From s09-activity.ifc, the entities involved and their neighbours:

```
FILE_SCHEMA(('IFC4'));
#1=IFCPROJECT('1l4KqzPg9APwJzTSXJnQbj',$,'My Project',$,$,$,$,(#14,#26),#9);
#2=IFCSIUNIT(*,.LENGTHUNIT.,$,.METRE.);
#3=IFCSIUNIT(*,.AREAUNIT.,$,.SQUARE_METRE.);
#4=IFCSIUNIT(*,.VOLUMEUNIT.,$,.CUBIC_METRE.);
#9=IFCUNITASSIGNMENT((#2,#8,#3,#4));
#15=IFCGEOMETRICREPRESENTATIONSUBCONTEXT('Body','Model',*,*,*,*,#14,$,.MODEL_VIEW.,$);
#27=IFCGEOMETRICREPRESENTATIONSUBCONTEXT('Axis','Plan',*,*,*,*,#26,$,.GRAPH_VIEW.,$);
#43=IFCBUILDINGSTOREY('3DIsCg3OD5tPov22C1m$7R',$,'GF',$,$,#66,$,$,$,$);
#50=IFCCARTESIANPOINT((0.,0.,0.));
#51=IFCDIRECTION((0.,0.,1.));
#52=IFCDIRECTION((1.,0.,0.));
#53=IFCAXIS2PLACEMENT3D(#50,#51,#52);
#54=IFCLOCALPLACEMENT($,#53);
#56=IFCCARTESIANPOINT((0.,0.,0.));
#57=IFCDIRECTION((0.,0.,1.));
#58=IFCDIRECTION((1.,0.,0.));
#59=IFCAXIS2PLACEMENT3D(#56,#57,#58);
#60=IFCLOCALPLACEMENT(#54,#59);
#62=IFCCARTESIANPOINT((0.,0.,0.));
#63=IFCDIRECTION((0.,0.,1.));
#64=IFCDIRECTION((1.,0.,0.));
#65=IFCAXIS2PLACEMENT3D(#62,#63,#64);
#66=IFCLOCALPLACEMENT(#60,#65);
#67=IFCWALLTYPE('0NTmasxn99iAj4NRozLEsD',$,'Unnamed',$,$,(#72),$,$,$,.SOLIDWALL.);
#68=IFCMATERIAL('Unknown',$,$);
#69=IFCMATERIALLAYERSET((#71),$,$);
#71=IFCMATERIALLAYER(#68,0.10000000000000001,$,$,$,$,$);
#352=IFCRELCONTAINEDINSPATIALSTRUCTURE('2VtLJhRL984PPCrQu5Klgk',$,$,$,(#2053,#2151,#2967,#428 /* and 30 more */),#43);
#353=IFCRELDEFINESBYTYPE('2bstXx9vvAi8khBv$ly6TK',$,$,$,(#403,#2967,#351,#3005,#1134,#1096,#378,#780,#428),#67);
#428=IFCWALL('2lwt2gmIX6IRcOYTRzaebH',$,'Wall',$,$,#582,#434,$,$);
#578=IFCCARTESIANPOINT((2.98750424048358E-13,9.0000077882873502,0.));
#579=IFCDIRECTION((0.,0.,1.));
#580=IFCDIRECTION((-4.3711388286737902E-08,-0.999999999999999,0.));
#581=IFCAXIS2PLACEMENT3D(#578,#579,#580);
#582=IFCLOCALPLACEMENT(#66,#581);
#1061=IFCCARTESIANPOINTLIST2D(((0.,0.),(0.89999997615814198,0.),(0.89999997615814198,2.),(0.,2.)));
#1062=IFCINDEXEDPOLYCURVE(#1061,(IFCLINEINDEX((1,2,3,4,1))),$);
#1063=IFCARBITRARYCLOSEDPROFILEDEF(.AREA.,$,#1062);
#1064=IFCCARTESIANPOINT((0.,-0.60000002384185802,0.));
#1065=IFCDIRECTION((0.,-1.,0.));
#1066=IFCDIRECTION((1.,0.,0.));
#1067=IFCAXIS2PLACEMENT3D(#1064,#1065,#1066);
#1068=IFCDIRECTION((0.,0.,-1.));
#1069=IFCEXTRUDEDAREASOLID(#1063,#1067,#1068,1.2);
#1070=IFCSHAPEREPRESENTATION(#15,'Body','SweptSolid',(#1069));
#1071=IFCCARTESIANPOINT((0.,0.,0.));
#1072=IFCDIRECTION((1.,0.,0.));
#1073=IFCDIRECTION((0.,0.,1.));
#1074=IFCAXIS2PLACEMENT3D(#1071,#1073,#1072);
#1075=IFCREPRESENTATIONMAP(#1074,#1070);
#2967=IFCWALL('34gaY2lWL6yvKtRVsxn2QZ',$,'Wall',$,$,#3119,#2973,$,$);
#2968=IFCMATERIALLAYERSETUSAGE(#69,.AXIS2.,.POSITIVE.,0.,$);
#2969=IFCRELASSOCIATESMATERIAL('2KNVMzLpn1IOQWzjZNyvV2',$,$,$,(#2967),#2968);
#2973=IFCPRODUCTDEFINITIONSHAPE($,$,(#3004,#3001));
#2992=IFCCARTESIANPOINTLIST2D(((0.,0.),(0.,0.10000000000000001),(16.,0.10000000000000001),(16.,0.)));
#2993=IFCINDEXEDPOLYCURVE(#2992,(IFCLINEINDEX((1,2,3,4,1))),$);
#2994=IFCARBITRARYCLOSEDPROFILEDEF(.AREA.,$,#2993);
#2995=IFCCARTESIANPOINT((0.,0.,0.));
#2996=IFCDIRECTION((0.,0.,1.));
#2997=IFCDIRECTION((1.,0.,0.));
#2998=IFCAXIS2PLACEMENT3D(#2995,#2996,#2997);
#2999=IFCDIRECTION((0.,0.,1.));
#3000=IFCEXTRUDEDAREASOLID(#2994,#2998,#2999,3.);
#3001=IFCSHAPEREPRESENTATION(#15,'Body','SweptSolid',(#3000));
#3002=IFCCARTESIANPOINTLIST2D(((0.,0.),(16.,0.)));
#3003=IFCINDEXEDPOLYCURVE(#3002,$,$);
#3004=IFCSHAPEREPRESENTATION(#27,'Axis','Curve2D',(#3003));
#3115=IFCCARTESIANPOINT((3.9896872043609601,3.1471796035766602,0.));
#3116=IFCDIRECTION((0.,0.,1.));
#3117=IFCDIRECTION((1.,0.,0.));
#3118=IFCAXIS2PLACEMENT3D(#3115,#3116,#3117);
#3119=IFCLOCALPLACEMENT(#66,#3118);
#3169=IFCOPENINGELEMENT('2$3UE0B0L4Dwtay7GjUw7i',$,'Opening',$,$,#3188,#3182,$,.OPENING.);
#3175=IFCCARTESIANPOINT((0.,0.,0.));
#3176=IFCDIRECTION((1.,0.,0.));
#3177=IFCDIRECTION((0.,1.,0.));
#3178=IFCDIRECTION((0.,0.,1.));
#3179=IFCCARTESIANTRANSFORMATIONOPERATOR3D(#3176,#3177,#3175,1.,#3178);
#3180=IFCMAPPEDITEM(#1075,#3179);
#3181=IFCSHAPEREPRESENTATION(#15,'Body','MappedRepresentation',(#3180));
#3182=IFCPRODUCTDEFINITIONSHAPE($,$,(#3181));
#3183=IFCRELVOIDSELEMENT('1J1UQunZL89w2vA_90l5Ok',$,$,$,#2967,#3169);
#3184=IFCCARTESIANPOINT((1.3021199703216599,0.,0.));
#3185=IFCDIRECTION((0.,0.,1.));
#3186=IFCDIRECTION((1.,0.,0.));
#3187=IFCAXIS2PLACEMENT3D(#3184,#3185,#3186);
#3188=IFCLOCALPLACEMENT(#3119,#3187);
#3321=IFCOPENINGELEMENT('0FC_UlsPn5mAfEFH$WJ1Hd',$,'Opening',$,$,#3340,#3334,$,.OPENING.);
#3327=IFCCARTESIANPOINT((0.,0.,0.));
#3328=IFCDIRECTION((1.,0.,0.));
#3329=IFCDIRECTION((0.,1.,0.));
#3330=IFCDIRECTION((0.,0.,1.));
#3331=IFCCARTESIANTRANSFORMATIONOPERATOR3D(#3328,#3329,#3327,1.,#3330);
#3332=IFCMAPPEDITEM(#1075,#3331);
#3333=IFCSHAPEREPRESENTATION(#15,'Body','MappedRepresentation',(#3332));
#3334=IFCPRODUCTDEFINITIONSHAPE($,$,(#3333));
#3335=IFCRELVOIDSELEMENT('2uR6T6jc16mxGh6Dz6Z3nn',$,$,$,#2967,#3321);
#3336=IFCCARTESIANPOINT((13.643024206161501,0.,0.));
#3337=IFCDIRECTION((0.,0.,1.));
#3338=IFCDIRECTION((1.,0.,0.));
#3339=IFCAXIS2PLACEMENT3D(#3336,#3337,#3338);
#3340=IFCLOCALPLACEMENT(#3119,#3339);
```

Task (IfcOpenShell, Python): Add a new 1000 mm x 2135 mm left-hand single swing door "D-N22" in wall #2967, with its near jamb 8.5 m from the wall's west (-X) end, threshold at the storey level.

```python
import numpy as np
import ifcopenshell
import ifcopenshell.api.feature
import ifcopenshell.api.geometry
import ifcopenshell.api.root
import ifcopenshell.api.spatial
import ifcopenshell.geom
import ifcopenshell.util.element
import ifcopenshell.util.placement
import ifcopenshell.util.representation
import ifcopenshell.util.shape
import ifcopenshell.util.unit

model = ifcopenshell.open("s09-activity.ifc")
unit_scale = ifcopenshell.util.unit.calculate_unit_scale(model)
settings = ifcopenshell.geom.settings()


def volume(element):
    """Net volume in cubic metres, openings subtracted."""
    shape = ifcopenshell.geom.create_shape(settings, element)
    return ifcopenshell.util.shape.get_volume(shape.geometry)


wall = model.by_guid("34gaY2lWL6yvKtRVsxn2QZ")
storey = ifcopenshell.util.element.get_container(wall, ifc_class="IfcBuildingStorey")
context = ifcopenshell.util.representation.get_context(model, "Model", "Body", "MODEL_VIEW")
before = volume(wall)

width, height, from_end, sill = 1, 2.135, 8.5, 0.0  # metres

# The wall runs along its own X axis, and the end named is its -X end.
wall_shape = ifcopenshell.geom.create_shape(settings, wall)
x, y, z = ifcopenshell.util.shape.get_vertices(wall_shape.geometry).T
start = x.min() + from_end
face, thickness = float(y.min()), float(y.max() - y.min())
wall_matrix = ifcopenshell.util.placement.get_local_placement(wall.ObjectPlacement)
level = ifcopenshell.util.placement.get_local_placement(storey.ObjectPlacement)[2, 3]


def in_wall(x, y):
    """Placement at x, y metres in the wall's axes, at sill height."""
    matrix = wall_matrix.copy()
    matrix[:, 3] = wall_matrix @ np.array([x / unit_scale, y / unit_scale, 0.0, 1.0])
    matrix[2, 3] = level + sill / unit_scale
    return matrix


# Opening: a box that overshoots both wall faces by 50 mm.
opening = ifcopenshell.api.root.create_entity(model, ifc_class="IfcOpeningElement", predefined_type="OPENING")
box = ifcopenshell.api.geometry.add_wall_representation(
    model, context=context, length=width, height=height, thickness=thickness + 0.1
)
ifcopenshell.api.geometry.assign_representation(model, product=opening, representation=box)
ifcopenshell.api.geometry.edit_object_placement(model, product=opening, matrix=in_wall(start, face - 0.05), is_si=False)
ifcopenshell.api.feature.add_feature(model, feature=opening, element=wall)

door = ifcopenshell.api.root.create_entity(model, ifc_class="IfcDoor", name="D-N22", predefined_type="DOOR")
door.OverallWidth, door.OverallHeight = width / unit_scale, height / unit_scale
door.OperationType = "SINGLE_SWING_LEFT"
body = ifcopenshell.api.geometry.add_door_representation(
    model,
    context=context,
    overall_width=door.OverallWidth,
    overall_height=door.OverallHeight,
    operation_type="SINGLE_SWING_LEFT",
    lining_properties={"LiningDepth": thickness / unit_scale, "ThresholdDepth": thickness / unit_scale},
)
ifcopenshell.api.geometry.assign_representation(model, product=door, representation=body)
ifcopenshell.api.spatial.assign_container(model, products=[door], relating_structure=storey)
ifcopenshell.api.feature.add_filling(model, opening=opening, element=door)

# The lining spans the wall, so the door starts at the wall face.
ifcopenshell.api.geometry.edit_object_placement(model, product=door, matrix=in_wall(start, face), is_si=False)

after = volume(wall)

print(f"wall volume {before:.3f} -> {after:.3f} m3")

model.write("s09-activity-out.ifc")
```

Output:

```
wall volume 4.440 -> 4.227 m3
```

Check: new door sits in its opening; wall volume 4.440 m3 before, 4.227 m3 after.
